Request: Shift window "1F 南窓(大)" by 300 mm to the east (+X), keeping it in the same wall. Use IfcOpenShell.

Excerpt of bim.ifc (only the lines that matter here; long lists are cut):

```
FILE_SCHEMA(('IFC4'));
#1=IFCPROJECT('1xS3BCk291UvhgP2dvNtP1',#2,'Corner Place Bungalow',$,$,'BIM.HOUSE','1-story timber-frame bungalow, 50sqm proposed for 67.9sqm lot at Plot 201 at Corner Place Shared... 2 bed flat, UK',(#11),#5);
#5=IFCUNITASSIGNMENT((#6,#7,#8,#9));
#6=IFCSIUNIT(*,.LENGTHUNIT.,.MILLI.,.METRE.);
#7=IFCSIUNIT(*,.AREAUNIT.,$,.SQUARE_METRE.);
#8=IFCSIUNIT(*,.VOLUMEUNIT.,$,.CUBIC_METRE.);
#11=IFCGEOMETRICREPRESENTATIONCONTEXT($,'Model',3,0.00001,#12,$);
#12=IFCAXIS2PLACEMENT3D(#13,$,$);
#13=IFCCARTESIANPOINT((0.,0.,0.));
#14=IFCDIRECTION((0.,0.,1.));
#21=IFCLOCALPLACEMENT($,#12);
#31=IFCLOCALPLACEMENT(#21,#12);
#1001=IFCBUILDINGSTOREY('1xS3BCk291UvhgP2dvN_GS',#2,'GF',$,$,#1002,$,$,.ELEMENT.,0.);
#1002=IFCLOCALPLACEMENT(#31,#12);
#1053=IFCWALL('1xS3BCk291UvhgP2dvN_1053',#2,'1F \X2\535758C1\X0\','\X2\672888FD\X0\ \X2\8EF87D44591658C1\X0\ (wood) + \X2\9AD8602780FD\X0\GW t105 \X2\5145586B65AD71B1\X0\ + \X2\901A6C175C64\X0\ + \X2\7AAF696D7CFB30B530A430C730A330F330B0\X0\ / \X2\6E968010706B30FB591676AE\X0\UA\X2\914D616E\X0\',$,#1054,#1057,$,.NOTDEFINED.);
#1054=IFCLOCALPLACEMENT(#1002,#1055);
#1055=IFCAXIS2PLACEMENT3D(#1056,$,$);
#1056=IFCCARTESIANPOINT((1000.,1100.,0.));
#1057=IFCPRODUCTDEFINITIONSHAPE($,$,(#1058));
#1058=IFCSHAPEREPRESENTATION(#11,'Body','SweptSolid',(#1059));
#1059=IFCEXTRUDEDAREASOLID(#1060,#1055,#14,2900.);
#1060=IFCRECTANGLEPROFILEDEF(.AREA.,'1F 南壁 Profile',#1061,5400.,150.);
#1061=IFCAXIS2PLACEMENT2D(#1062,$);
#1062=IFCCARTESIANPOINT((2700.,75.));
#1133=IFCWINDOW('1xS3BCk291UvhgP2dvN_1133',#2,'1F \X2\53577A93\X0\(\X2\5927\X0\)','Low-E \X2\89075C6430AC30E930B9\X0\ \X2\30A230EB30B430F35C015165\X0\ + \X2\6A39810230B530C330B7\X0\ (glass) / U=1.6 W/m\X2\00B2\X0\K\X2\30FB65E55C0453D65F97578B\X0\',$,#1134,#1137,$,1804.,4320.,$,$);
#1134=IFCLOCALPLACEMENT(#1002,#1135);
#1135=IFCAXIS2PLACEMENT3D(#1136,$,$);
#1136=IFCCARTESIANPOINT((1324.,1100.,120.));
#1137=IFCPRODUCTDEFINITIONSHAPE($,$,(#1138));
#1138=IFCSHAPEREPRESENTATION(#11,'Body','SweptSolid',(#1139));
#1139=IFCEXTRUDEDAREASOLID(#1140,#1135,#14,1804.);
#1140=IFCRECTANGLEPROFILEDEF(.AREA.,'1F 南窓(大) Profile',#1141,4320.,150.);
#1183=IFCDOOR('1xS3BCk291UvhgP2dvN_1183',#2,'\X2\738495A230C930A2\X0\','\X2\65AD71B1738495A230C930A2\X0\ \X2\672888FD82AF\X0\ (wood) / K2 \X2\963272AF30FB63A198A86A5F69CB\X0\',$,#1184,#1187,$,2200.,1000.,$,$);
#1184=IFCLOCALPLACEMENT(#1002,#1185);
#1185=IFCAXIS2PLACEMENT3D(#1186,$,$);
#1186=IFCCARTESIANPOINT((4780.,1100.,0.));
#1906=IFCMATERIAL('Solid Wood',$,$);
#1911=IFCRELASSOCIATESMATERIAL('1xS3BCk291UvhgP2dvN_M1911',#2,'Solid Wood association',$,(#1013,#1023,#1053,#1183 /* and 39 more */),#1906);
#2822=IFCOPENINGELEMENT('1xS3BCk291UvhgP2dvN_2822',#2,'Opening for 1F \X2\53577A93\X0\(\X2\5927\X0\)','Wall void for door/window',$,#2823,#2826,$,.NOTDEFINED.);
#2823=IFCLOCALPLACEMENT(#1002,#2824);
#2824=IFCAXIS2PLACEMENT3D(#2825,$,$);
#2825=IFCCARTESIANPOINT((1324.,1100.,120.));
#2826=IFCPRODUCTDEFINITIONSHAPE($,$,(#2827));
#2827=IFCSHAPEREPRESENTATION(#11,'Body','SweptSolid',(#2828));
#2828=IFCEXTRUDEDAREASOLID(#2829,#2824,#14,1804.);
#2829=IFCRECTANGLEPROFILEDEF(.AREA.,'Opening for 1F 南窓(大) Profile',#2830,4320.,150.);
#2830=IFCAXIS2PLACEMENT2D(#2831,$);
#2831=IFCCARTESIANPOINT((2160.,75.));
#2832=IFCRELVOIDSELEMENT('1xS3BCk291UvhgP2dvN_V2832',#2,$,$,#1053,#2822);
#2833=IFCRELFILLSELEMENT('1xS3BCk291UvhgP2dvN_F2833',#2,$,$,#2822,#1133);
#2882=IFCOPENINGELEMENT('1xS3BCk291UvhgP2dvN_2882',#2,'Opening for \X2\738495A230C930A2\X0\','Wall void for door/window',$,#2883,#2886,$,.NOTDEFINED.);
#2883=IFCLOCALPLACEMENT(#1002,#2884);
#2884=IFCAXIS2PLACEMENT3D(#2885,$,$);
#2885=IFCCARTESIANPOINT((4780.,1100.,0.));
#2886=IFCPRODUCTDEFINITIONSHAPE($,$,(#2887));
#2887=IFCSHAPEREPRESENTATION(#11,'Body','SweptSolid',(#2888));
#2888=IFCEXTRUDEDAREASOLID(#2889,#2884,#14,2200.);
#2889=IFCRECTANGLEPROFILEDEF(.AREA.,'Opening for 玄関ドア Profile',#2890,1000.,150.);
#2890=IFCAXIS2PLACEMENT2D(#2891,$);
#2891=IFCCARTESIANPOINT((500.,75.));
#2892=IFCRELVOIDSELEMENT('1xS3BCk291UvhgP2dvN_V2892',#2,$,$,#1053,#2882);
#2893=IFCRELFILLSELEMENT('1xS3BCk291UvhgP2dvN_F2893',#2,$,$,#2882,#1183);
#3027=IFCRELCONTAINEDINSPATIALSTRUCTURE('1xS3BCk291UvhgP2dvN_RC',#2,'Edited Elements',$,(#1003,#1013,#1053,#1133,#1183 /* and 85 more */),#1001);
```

```python
import ifcopenshell
import ifcopenshell.api.geometry
import ifcopenshell.util.placement

model = ifcopenshell.open("bim.ifc")

window = model.by_guid("1xS3BCk291UvhgP2dvN_1133")
opening = window.FillsVoids[0].RelatingOpeningElement
wall = opening.VoidsElements[0].RelatingBuildingElement

wall_matrix = ifcopenshell.util.placement.get_local_placement(wall.ObjectPlacement)
shift = wall_matrix[:3, 0] * 300.0
before = ifcopenshell.util.placement.get_local_placement(window.ObjectPlacement)[:3, 3].copy()

# The window is not placed relative to its opening, so move both.
for product in (opening, window):
    matrix = ifcopenshell.util.placement.get_local_placement(product.ObjectPlacement)
    matrix[:3, 3] += shift
    ifcopenshell.api.geometry.edit_object_placement(model, product=product, matrix=matrix, is_si=False)

after = ifcopenshell.util.placement.get_local_placement(window.ObjectPlacement)[:3, 3]
print("window moved by", (after - before).round(3) + 0.0)

model.write("bim_edited.ifc")
```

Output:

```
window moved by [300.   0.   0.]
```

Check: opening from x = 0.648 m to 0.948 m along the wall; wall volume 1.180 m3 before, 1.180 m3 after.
